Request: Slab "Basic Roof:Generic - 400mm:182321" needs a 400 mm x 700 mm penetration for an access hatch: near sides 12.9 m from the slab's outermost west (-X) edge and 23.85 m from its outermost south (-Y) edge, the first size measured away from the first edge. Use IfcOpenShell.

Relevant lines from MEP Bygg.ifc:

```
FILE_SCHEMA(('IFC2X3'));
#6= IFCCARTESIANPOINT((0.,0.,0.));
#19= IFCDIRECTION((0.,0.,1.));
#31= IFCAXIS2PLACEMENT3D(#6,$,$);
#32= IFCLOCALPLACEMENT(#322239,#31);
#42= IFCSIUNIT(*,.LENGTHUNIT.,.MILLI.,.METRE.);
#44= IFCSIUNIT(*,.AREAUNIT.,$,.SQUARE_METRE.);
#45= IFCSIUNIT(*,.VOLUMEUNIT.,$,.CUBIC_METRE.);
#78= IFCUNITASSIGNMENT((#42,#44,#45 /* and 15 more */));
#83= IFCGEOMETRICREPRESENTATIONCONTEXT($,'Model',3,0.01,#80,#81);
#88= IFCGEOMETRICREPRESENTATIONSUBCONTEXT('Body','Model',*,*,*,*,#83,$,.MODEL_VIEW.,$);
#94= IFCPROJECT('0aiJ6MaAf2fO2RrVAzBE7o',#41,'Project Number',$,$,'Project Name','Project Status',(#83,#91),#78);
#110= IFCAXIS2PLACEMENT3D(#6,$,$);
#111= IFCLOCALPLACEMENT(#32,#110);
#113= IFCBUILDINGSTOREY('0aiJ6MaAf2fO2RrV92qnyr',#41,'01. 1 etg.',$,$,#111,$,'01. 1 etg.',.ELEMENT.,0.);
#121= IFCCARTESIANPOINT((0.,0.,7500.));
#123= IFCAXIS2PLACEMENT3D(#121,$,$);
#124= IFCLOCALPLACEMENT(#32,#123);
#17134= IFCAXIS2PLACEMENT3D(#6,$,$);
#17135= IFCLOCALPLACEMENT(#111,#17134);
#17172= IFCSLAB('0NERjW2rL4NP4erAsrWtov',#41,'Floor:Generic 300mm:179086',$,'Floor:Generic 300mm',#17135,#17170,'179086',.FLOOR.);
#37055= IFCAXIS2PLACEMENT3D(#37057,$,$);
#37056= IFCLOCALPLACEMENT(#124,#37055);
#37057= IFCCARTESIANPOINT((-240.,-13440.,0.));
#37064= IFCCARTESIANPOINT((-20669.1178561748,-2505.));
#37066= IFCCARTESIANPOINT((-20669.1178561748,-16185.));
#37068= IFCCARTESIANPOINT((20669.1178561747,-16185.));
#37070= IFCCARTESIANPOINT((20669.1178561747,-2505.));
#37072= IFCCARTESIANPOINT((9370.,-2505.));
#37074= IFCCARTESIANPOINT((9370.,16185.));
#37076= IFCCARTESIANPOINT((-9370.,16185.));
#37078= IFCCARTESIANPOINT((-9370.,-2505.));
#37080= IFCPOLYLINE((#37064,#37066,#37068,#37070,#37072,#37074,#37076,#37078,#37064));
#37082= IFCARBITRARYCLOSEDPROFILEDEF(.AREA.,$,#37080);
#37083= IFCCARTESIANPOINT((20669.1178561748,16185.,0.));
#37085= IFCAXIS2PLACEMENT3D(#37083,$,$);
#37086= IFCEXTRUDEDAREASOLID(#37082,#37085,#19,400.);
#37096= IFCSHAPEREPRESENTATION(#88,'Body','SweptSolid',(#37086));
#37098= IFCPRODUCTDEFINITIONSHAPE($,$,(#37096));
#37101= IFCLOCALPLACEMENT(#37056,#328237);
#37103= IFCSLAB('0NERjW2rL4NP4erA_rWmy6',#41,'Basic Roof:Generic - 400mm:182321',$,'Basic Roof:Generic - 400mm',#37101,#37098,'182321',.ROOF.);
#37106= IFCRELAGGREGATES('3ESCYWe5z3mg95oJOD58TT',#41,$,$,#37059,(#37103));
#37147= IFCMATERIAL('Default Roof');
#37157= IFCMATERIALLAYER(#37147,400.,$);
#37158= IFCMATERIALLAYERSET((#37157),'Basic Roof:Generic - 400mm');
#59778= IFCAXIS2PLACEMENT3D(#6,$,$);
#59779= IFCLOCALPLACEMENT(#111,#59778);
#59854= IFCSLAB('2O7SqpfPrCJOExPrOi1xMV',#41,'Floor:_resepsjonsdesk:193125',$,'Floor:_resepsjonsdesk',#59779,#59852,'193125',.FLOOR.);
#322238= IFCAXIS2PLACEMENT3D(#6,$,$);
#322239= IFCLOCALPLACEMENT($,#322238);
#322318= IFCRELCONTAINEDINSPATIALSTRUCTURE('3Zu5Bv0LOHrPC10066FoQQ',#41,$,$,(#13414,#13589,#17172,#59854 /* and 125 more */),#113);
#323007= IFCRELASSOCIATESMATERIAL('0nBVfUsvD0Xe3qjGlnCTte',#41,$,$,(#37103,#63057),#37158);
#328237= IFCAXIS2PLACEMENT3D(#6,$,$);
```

```python
import numpy as np
import ifcopenshell
import ifcopenshell.api.feature
import ifcopenshell.api.geometry
import ifcopenshell.api.root
import ifcopenshell.geom
import ifcopenshell.util.placement
import ifcopenshell.util.representation
import ifcopenshell.util.shape
import ifcopenshell.util.unit

model = ifcopenshell.open("MEP Bygg.ifc")
unit_scale = ifcopenshell.util.unit.calculate_unit_scale(model)
settings = ifcopenshell.geom.settings()


def volume(element):
    """Net volume in cubic metres, openings subtracted."""
    shape = ifcopenshell.geom.create_shape(settings, element)
    return ifcopenshell.util.shape.get_volume(shape.geometry)


slab = model.by_guid("0NERjW2rL4NP4erA_rWmy6")
before = volume(slab)

# Extent in the slab's own axes, in metres. The edges named are its -X and -Y sides.
slab_shape = ifcopenshell.geom.create_shape(settings, slab)
vertices = ifcopenshell.util.shape.get_vertices(slab_shape.geometry)
x_min, y_min, bottom = vertices.min(axis=0)
top = vertices[:, 2].max()

opening = ifcopenshell.api.root.create_entity(model, ifc_class="IfcOpeningElement", name="Access hatch opening")
context = ifcopenshell.util.representation.get_context(model, "Model", "Body", "MODEL_VIEW")
width, depth = 0.4, 0.7
outline = [(0.0, 0.0), (width, 0.0), (width, depth), (0.0, depth), (0.0, 0.0)]
# Overshoot both faces by 50 mm so the cut is clean.
shape = ifcopenshell.api.geometry.add_slab_representation(
    model, context=context, depth=top - bottom + 0.1, polyline=outline
)
ifcopenshell.api.geometry.assign_representation(model, product=opening, representation=shape)

matrix = ifcopenshell.util.placement.get_local_placement(slab.ObjectPlacement)
matrix[:, 3] = matrix @ np.append(np.array([x_min + 12.9, y_min + 23.85, bottom - 0.05]) / unit_scale, 1.0)
ifcopenshell.api.geometry.edit_object_placement(model, product=opening, matrix=matrix, is_si=False)
ifcopenshell.api.feature.add_feature(model, feature=opening, element=slab)

after = volume(slab)

print(f"slab volume {before:.3f} -> {after:.3f} m3")

model.write("MEP Bygg_v2.ifc")
```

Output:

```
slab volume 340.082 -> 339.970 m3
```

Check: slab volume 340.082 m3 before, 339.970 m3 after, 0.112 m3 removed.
